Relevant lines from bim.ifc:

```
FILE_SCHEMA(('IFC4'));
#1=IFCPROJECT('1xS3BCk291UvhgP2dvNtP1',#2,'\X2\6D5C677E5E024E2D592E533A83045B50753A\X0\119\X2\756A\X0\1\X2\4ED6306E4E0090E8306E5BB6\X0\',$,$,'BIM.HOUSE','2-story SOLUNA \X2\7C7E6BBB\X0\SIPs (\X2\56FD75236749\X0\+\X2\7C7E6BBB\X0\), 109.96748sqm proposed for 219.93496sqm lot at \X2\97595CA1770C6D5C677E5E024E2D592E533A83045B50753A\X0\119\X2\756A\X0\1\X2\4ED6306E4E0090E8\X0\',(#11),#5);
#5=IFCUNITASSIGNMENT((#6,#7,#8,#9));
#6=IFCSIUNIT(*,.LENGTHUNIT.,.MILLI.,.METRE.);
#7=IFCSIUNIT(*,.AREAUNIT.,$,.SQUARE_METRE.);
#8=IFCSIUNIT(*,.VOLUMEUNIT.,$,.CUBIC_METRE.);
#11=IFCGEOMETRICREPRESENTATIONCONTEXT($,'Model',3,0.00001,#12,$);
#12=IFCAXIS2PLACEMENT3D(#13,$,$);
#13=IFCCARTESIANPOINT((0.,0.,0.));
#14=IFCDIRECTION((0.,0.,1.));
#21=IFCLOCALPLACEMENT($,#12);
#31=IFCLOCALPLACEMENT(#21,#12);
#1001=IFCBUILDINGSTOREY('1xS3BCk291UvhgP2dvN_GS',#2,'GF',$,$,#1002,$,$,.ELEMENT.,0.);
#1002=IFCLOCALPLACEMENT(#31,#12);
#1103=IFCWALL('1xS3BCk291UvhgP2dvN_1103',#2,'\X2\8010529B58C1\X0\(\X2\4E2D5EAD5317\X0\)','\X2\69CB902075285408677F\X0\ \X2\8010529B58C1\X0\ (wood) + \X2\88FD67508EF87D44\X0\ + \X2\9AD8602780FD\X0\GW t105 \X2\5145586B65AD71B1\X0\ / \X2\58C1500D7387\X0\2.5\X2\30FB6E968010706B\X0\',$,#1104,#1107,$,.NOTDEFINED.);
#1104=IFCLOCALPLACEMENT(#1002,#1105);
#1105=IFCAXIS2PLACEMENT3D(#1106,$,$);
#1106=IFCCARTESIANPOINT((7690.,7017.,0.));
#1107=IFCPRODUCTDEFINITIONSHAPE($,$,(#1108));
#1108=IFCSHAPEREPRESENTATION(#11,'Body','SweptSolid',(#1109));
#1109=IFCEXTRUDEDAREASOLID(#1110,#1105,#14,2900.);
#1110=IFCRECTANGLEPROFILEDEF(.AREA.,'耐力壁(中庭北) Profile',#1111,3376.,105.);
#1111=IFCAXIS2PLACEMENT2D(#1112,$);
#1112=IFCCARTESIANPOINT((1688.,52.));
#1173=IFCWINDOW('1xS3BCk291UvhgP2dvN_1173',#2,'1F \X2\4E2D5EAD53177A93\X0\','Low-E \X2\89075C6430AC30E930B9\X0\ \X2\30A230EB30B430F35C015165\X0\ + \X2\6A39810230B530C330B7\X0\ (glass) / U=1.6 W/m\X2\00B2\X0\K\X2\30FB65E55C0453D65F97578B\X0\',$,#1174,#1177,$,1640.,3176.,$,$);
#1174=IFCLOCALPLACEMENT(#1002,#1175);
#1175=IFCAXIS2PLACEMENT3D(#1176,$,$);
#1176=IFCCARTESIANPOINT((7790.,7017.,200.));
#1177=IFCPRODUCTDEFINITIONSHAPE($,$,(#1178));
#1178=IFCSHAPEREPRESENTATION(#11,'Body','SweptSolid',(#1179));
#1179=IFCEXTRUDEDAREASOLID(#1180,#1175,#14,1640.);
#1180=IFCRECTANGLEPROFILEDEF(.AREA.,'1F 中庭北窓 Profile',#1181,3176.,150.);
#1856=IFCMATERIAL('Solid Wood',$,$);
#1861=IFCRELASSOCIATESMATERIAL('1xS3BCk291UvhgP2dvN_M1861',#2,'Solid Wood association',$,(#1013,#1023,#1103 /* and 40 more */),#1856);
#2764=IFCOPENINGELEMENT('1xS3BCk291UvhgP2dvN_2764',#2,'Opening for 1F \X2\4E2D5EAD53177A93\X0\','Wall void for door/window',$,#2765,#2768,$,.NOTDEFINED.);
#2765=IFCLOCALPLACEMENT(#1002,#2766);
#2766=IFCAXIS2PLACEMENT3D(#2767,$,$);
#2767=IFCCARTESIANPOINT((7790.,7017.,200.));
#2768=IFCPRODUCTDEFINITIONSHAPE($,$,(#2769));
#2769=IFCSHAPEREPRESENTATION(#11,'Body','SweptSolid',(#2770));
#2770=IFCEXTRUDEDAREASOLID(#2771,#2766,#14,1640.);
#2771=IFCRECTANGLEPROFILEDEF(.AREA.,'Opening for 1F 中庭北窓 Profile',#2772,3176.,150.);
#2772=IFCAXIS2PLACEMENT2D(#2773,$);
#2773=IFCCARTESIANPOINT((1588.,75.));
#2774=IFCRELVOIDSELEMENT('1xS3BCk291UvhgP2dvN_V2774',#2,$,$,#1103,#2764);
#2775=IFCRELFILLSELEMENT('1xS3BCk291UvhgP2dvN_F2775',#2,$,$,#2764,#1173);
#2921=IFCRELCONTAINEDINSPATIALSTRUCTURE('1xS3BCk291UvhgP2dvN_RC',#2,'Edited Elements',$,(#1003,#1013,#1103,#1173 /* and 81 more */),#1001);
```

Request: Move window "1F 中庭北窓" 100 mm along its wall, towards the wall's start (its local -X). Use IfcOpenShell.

```python
import ifcopenshell
import ifcopenshell.api.geometry
import ifcopenshell.util.placement

model = ifcopenshell.open("bim.ifc")

window = model.by_guid("1xS3BCk291UvhgP2dvN_1173")
opening = window.FillsVoids[0].RelatingOpeningElement
wall = opening.VoidsElements[0].RelatingBuildingElement

wall_matrix = ifcopenshell.util.placement.get_local_placement(wall.ObjectPlacement)
shift = wall_matrix[:3, 0] * -100.0
before = ifcopenshell.util.placement.get_local_placement(window.ObjectPlacement)[:3, 3].copy()

# The window is not placed relative to its opening, so move both.
for product in (opening, window):
    matrix = ifcopenshell.util.placement.get_local_placement(product.ObjectPlacement)
    matrix[:3, 3] += shift
    ifcopenshell.api.geometry.edit_object_placement(model, product=product, matrix=matrix, is_si=False)

after = ifcopenshell.util.placement.get_local_placement(window.ObjectPlacement)[:3, 3]
print("window moved by", (after - before).round(3) + 0.0)

model.write("bim_updated.ifc")
```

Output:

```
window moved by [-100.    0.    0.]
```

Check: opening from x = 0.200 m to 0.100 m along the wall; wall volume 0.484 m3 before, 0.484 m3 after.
